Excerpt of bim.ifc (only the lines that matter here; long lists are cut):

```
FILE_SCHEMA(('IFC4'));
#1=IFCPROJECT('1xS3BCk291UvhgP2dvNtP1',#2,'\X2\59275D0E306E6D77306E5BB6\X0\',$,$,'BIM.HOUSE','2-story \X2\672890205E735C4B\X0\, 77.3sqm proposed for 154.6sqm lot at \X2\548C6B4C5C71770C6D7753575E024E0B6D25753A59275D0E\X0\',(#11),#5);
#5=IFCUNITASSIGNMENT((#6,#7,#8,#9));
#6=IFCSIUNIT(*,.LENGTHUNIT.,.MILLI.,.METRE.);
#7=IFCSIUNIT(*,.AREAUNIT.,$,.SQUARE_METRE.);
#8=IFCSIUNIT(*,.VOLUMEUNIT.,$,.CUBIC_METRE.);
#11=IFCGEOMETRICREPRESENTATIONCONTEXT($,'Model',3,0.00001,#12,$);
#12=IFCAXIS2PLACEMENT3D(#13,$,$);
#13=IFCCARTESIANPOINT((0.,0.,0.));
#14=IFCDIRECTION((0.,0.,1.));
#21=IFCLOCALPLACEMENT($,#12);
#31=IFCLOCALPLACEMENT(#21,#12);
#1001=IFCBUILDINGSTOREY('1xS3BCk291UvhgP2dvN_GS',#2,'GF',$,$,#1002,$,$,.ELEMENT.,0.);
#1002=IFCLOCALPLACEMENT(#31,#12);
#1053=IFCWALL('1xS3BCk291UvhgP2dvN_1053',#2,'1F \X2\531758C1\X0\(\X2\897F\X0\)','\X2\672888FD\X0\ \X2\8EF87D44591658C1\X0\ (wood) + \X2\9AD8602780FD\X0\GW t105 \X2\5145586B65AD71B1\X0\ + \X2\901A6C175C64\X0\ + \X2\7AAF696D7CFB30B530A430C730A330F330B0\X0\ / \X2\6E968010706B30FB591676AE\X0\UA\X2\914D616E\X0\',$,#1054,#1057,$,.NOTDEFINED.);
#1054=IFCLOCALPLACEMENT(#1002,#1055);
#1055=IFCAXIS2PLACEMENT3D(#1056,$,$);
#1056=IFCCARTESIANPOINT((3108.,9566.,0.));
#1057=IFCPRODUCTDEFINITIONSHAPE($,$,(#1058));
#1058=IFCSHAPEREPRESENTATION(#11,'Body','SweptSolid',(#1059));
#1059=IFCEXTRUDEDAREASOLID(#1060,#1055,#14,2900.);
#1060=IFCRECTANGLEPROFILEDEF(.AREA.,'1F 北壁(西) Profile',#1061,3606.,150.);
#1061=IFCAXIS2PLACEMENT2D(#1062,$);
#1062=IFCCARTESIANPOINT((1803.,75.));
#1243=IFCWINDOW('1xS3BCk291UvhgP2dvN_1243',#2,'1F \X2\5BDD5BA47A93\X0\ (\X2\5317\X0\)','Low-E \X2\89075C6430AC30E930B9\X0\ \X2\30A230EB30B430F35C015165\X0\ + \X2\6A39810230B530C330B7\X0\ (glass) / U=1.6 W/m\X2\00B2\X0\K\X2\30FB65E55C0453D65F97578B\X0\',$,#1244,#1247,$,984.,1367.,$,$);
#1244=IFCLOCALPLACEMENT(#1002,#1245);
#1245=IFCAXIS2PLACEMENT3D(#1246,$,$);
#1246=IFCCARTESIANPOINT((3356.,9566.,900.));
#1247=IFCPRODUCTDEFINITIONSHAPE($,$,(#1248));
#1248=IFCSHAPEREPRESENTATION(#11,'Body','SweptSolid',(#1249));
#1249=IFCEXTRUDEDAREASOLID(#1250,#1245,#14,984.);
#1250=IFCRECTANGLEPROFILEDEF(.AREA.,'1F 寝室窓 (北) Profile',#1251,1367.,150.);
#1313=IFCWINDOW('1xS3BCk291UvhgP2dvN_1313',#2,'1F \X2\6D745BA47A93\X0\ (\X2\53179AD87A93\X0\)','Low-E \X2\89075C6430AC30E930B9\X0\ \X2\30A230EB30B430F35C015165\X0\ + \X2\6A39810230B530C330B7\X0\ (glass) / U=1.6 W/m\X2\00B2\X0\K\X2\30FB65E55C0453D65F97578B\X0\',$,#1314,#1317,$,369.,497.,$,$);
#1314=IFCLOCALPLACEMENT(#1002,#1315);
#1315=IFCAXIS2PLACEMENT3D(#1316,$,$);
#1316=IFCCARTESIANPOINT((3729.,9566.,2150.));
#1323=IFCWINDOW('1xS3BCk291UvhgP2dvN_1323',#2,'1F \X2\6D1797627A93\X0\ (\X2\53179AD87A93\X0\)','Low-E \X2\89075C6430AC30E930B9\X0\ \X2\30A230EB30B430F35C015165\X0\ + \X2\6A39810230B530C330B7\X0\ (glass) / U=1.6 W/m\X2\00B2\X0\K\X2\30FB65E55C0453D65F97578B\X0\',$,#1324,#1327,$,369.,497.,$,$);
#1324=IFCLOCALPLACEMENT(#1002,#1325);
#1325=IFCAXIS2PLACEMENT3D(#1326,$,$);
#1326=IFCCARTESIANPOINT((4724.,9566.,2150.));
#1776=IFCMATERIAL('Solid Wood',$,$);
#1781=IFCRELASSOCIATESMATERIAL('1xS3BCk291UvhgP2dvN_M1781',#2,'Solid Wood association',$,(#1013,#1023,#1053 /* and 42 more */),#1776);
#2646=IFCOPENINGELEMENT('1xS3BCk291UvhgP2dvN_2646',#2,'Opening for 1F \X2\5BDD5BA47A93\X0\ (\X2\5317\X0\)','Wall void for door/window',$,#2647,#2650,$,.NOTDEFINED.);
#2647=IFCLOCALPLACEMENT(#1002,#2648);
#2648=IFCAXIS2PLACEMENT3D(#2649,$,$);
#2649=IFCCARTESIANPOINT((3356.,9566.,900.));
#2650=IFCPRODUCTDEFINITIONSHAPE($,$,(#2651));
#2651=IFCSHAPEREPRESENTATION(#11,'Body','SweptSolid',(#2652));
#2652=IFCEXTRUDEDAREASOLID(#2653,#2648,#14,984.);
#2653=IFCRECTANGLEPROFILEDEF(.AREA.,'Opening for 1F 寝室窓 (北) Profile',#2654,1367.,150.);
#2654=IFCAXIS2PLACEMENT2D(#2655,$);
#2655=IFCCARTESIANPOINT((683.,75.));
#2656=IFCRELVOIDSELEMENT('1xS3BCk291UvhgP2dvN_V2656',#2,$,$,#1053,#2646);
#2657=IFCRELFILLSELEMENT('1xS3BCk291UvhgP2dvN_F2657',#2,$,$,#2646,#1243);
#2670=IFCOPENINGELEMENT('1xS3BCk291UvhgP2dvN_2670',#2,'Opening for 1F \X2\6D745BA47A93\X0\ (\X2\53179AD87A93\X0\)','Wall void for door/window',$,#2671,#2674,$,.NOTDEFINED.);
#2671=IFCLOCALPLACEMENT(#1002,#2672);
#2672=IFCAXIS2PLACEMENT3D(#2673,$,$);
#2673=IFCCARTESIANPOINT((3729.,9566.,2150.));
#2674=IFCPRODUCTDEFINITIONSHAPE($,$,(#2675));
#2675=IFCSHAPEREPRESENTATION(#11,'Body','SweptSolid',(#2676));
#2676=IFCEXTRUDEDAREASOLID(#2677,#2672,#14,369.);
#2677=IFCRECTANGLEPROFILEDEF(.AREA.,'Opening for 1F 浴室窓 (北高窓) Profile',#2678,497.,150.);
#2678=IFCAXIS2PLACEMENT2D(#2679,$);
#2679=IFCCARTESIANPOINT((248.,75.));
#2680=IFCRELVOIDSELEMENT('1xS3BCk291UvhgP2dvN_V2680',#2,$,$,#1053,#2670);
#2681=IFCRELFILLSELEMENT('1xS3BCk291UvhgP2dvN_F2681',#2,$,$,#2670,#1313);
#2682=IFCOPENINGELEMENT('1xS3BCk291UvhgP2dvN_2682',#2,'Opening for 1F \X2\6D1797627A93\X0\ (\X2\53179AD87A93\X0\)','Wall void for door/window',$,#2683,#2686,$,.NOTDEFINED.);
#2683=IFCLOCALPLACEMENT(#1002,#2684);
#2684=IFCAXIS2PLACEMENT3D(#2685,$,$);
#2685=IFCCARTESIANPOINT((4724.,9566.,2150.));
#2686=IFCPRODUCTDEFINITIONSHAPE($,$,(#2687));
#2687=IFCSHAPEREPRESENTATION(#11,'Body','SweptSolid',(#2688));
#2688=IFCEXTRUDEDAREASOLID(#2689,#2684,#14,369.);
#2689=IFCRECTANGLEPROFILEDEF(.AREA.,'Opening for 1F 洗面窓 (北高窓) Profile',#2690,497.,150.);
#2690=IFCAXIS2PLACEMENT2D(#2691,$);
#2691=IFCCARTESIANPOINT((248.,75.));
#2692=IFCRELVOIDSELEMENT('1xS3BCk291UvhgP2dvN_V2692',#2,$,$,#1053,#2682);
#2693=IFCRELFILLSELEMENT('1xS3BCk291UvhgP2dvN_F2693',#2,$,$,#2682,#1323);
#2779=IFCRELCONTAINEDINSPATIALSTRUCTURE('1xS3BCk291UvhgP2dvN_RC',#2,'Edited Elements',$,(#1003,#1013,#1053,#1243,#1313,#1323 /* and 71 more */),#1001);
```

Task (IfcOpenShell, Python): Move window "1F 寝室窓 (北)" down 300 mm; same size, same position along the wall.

```python
import numpy as np
import ifcopenshell
import ifcopenshell.api.geometry
import ifcopenshell.util.placement
import ifcopenshell.util.unit

model = ifcopenshell.open("bim.ifc")
unit_scale = ifcopenshell.util.unit.calculate_unit_scale(model)

window = model.by_id(1243)
opening = window.FillsVoids[0].RelatingOpeningElement
dz = -300.0

shift = np.array([0.0, 0.0, dz])
# The window is not placed relative to its opening, so move both.
for product in (opening, window):
    matrix = ifcopenshell.util.placement.get_local_placement(product.ObjectPlacement)
    matrix[:3, 3] += shift
    ifcopenshell.api.geometry.edit_object_placement(model, product=product, matrix=matrix, is_si=False)

print(f"moved by {dz * unit_scale:+.3f} m")

model.write("bim-out.ifc")
```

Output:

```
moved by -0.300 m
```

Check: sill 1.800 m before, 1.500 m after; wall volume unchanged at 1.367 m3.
